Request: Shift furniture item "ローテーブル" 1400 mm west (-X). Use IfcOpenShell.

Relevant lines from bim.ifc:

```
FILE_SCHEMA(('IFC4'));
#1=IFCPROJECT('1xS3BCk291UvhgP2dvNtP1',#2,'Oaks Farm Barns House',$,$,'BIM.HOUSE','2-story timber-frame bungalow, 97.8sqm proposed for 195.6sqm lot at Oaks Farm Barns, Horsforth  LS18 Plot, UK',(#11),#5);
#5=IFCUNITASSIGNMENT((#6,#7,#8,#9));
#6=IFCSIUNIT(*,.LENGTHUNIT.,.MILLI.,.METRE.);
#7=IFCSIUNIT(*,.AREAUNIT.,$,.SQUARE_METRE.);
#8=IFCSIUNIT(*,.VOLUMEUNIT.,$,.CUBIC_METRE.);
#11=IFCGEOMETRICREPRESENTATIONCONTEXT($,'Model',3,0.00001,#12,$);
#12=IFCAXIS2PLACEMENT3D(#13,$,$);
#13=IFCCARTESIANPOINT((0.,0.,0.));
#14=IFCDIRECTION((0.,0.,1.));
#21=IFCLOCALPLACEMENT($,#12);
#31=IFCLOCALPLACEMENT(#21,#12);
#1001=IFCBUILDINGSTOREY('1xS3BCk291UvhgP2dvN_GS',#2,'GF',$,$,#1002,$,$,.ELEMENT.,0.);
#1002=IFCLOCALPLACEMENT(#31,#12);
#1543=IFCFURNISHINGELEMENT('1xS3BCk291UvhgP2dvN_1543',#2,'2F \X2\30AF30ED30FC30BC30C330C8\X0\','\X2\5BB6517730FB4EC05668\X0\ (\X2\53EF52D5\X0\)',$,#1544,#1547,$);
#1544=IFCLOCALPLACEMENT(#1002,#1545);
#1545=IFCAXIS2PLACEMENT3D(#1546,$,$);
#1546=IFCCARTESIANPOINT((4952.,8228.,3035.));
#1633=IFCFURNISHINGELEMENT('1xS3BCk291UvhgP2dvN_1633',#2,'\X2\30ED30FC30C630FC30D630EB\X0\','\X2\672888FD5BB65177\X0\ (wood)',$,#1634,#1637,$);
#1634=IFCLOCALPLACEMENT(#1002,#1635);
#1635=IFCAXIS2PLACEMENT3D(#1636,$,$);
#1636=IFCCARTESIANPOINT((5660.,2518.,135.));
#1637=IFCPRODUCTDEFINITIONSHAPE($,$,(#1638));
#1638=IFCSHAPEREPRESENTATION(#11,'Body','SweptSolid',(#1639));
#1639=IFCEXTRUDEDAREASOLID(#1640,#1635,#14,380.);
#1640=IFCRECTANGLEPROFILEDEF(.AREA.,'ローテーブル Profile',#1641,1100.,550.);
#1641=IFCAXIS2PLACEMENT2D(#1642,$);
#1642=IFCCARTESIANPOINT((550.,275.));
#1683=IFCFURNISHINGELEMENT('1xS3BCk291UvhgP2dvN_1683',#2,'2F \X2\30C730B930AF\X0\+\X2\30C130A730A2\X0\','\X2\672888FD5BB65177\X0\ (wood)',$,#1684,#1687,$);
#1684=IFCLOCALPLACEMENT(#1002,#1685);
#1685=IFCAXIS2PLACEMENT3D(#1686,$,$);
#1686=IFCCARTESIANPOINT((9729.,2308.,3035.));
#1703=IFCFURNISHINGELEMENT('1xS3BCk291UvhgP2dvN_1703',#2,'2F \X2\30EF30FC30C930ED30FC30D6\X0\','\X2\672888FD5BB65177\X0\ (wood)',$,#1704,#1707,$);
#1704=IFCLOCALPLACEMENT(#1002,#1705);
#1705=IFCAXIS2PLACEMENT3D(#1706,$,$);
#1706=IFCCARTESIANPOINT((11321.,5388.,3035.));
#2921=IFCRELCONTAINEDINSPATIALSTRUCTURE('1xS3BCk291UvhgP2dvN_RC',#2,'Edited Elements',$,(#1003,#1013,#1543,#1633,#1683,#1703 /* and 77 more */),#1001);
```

```python
import ifcopenshell
import ifcopenshell.api.geometry
import ifcopenshell.util.placement
import ifcopenshell.util.unit

model = ifcopenshell.open("bim.ifc")
unit_scale = ifcopenshell.util.unit.calculate_unit_scale(model)

item = model.by_id(1633)
matrix = ifcopenshell.util.placement.get_local_placement(item.ObjectPlacement)
matrix[0, 3] -= 1.4 / unit_scale
ifcopenshell.api.geometry.edit_object_placement(model, product=item, matrix=matrix, is_si=False)

print(ifcopenshell.util.placement.get_local_placement(item.ObjectPlacement).round(3) + 0.0)

model.write("bim_v2.ifc")
```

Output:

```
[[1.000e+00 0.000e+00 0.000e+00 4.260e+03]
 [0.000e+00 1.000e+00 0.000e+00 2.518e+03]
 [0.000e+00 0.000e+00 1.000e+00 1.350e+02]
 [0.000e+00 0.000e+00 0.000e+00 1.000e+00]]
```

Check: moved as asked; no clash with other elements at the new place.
